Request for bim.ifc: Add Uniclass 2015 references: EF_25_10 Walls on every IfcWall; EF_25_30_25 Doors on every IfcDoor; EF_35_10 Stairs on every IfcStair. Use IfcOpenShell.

First a look at what the model holds.

```python
import ifcopenshell

model = ifcopenshell.open("bim.ifc")
print(model.schema)
print("classifications:", [c.Name for c in model.by_type("IfcClassification")])
for ifc_class in ("IfcDoor", "IfcRoof", "IfcStair", "IfcWall", "IfcWindow"):
    print(ifc_class, len(model.by_type(ifc_class)))
```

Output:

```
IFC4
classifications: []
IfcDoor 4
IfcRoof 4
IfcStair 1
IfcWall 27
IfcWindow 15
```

```python
import ifcopenshell
import ifcopenshell.api.classification

model = ifcopenshell.open("bim.ifc")

system = ifcopenshell.api.classification.add_classification(model, classification="Uniclass 2015")

codes = {
    "IfcWall": ("EF_25_10", "Walls"),
    "IfcDoor": ("EF_25_30_25", "Doors"),
    "IfcStair": ("EF_35_10", "Stairs"),
}
for ifc_class, (code, name) in codes.items():
    products = model.by_type(ifc_class)
    ifcopenshell.api.classification.add_reference(
        model, products=products, classification=system, identification=code, name=name
    )
    print(code, len(products))

model.write("bim_v2.ifc")
```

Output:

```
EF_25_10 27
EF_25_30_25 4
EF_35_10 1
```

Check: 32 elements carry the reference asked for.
